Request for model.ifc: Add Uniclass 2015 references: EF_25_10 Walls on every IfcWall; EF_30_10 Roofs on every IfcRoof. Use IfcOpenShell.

First a look at what the model holds.

```python
import ifcopenshell

model = ifcopenshell.open("model.ifc")
print(model.schema)
print("classifications:", [c.Name for c in model.by_type("IfcClassification")])
for ifc_class in ("IfcDoor", "IfcRoof", "IfcStair", "IfcWall", "IfcWindow"):
    print(ifc_class, len(model.by_type(ifc_class)))
```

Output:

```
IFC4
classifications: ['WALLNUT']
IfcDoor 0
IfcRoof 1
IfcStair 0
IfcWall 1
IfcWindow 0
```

```python
import ifcopenshell
import ifcopenshell.api.classification

model = ifcopenshell.open("model.ifc")

system = ifcopenshell.api.classification.add_classification(model, classification="Uniclass 2015")

codes = {
    "IfcWall": ("EF_25_10", "Walls"),
    "IfcRoof": ("EF_30_10", "Roofs"),
}
for ifc_class, (code, name) in codes.items():
    products = model.by_type(ifc_class)
    ifcopenshell.api.classification.add_reference(
        model, products=products, classification=system, identification=code, name=name
    )
    print(code, len(products))

model.write("model_edited.ifc")
```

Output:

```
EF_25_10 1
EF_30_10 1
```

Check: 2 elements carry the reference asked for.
